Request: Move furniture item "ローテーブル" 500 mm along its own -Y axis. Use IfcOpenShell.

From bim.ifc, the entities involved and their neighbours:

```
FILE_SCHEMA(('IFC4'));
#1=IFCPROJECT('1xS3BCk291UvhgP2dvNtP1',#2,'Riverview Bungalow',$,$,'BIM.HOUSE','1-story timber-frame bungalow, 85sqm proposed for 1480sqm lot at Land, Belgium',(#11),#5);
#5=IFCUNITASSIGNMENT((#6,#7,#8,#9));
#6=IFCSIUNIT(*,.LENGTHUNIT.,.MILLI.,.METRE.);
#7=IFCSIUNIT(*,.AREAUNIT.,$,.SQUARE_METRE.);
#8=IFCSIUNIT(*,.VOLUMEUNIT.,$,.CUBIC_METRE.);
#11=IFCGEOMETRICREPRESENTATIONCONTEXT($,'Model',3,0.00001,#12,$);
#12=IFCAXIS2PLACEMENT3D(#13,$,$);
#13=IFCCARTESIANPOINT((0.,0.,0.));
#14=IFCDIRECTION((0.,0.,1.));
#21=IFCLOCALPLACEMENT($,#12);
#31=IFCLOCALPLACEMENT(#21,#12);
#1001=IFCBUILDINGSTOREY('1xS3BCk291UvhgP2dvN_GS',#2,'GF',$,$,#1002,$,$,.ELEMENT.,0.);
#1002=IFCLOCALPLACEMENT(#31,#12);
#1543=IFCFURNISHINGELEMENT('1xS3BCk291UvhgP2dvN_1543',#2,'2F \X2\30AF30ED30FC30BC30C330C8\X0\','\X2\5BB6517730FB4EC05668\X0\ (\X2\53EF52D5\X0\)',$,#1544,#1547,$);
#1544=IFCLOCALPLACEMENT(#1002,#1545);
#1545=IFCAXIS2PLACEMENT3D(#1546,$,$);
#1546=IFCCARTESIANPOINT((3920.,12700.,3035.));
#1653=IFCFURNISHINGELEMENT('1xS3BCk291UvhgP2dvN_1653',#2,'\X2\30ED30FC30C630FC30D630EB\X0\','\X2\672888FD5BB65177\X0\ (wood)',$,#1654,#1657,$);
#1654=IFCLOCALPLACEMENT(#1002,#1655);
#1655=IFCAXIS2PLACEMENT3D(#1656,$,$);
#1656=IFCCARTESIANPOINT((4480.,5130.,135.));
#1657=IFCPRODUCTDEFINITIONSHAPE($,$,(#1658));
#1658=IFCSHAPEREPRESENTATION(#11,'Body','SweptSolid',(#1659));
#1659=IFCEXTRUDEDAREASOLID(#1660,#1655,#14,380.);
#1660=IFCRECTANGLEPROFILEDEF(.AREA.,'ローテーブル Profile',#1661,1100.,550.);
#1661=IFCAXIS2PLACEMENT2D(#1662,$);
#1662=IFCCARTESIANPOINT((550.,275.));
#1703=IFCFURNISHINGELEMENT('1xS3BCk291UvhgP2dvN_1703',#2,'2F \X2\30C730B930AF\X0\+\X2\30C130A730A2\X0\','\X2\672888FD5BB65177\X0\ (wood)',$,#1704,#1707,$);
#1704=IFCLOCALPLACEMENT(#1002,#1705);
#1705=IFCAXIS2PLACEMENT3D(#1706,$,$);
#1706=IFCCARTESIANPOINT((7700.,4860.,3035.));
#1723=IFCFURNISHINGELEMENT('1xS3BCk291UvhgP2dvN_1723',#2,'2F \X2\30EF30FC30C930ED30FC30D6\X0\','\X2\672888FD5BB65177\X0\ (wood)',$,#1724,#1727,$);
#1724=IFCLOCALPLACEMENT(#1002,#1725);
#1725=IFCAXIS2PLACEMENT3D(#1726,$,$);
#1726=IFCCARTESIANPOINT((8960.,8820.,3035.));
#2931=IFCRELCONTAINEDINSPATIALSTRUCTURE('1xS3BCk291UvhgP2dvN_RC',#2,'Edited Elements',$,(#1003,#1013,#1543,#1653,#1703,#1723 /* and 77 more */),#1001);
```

```python
import ifcopenshell
import ifcopenshell.api.geometry
import ifcopenshell.util.placement

model = ifcopenshell.open("bim.ifc")

item = model.by_id(1653)
matrix = ifcopenshell.util.placement.get_local_placement(item.ObjectPlacement)
matrix[:3, 3] -= matrix[:3, 1] * 500.0
ifcopenshell.api.geometry.edit_object_placement(model, product=item, matrix=matrix, is_si=False)

print(ifcopenshell.util.placement.get_local_placement(item.ObjectPlacement).round(3) + 0.0)

model.write("bim_edited.ifc")
```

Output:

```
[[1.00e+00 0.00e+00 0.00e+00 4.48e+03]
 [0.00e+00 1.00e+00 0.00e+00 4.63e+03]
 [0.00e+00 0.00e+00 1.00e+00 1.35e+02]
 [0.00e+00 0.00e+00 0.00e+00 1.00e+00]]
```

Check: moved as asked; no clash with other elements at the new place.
